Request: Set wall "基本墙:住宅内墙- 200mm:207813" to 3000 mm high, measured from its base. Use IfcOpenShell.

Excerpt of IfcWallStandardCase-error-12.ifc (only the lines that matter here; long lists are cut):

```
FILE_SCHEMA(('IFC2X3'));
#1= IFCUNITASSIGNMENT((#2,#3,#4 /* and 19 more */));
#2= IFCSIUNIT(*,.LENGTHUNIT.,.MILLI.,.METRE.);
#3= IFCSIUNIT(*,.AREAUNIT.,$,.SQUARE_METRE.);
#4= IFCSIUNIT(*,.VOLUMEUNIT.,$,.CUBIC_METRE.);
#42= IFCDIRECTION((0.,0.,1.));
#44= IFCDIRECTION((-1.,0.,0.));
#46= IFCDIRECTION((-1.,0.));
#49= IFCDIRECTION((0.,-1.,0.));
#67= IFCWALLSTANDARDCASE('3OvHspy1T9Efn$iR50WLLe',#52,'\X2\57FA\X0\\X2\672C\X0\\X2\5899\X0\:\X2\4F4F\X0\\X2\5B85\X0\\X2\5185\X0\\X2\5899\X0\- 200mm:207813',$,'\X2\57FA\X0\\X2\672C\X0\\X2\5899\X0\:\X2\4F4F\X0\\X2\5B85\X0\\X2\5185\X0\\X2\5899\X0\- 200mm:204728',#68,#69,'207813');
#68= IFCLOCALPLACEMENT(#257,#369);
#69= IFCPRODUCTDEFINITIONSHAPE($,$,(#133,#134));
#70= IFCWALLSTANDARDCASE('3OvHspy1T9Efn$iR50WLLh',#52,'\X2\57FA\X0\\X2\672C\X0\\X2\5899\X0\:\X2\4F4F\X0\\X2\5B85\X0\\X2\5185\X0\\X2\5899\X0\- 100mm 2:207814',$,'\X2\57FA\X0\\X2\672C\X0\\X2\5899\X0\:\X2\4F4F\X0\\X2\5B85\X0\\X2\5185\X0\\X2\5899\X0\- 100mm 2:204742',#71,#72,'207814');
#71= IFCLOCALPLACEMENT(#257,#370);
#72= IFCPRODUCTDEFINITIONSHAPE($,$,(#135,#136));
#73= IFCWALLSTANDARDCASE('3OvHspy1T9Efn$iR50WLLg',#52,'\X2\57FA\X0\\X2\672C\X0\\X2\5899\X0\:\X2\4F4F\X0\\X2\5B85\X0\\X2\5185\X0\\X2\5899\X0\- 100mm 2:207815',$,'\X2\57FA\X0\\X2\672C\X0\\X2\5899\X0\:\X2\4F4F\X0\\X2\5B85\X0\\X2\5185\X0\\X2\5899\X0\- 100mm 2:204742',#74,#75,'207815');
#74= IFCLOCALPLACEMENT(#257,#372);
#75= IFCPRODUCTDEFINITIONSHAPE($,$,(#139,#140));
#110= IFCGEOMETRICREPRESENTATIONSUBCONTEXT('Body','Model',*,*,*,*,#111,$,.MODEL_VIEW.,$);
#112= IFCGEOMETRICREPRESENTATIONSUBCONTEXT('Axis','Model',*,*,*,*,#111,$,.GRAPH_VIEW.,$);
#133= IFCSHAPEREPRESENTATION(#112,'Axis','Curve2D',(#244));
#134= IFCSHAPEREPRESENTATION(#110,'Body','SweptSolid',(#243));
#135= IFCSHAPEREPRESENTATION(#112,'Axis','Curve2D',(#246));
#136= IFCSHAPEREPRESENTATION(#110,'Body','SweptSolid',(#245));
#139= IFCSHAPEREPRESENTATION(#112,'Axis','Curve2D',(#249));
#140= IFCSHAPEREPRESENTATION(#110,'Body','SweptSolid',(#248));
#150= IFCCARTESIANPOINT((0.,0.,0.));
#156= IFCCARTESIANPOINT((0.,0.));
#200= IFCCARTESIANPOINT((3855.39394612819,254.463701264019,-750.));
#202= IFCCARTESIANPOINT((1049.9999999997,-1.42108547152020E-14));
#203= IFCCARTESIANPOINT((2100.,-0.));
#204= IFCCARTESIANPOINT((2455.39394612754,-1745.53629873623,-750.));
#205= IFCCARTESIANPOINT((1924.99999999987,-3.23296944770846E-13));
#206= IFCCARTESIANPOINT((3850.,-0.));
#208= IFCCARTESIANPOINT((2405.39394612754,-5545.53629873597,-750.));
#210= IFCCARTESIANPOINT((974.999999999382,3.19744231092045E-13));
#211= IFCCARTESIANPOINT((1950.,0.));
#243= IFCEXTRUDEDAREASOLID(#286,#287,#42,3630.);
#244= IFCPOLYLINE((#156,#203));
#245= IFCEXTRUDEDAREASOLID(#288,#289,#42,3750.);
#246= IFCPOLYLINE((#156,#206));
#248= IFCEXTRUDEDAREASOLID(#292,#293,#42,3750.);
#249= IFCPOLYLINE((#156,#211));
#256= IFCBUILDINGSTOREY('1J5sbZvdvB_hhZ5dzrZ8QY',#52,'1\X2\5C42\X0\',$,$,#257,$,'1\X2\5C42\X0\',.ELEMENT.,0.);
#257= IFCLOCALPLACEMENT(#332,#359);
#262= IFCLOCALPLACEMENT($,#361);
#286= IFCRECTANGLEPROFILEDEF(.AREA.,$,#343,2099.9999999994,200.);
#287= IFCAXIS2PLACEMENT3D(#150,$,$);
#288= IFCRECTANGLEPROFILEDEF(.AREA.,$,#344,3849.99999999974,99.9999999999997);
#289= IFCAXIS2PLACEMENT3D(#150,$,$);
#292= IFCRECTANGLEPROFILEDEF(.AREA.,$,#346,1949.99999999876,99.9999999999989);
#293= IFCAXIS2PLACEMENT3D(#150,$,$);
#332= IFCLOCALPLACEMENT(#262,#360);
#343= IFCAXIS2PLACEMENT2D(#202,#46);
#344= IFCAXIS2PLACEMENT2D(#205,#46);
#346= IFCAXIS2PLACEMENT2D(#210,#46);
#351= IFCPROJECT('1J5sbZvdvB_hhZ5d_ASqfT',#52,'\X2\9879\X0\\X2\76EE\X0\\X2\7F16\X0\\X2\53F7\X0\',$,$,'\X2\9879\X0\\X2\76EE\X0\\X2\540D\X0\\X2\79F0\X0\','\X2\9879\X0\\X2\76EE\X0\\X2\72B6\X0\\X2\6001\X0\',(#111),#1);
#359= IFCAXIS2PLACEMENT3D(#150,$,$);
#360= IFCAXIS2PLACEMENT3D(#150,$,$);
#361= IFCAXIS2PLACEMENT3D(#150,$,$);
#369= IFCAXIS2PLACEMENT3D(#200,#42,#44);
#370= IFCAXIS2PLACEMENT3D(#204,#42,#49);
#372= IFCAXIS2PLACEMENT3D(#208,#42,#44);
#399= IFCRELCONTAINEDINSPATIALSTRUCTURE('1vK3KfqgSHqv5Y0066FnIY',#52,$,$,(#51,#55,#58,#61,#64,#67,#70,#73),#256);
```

```python
import ifcopenshell
import ifcopenshell.geom
import ifcopenshell.util.representation
import ifcopenshell.util.shape

model = ifcopenshell.open("IfcWallStandardCase-error-12.ifc")
settings = ifcopenshell.geom.settings()


def volume(element):
    """Net volume in cubic metres, openings subtracted."""
    shape = ifcopenshell.geom.create_shape(settings, element)
    return ifcopenshell.util.shape.get_volume(shape.geometry)


wall = model.by_id(67)
before = volume(wall)

body = ifcopenshell.util.representation.get_representation(wall, "Model", "Body")
solid = body.Items[0]
old_height = solid.Depth
solid.Depth = 3000.0
after = volume(wall)

print(f"height {old_height:g} -> {solid.Depth:g}, volume {before:.3f} -> {after:.3f} m3")

model.write("IfcWallStandardCase-error-12_edited.ifc")
```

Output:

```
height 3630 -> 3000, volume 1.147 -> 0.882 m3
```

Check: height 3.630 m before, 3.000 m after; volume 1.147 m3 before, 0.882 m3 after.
